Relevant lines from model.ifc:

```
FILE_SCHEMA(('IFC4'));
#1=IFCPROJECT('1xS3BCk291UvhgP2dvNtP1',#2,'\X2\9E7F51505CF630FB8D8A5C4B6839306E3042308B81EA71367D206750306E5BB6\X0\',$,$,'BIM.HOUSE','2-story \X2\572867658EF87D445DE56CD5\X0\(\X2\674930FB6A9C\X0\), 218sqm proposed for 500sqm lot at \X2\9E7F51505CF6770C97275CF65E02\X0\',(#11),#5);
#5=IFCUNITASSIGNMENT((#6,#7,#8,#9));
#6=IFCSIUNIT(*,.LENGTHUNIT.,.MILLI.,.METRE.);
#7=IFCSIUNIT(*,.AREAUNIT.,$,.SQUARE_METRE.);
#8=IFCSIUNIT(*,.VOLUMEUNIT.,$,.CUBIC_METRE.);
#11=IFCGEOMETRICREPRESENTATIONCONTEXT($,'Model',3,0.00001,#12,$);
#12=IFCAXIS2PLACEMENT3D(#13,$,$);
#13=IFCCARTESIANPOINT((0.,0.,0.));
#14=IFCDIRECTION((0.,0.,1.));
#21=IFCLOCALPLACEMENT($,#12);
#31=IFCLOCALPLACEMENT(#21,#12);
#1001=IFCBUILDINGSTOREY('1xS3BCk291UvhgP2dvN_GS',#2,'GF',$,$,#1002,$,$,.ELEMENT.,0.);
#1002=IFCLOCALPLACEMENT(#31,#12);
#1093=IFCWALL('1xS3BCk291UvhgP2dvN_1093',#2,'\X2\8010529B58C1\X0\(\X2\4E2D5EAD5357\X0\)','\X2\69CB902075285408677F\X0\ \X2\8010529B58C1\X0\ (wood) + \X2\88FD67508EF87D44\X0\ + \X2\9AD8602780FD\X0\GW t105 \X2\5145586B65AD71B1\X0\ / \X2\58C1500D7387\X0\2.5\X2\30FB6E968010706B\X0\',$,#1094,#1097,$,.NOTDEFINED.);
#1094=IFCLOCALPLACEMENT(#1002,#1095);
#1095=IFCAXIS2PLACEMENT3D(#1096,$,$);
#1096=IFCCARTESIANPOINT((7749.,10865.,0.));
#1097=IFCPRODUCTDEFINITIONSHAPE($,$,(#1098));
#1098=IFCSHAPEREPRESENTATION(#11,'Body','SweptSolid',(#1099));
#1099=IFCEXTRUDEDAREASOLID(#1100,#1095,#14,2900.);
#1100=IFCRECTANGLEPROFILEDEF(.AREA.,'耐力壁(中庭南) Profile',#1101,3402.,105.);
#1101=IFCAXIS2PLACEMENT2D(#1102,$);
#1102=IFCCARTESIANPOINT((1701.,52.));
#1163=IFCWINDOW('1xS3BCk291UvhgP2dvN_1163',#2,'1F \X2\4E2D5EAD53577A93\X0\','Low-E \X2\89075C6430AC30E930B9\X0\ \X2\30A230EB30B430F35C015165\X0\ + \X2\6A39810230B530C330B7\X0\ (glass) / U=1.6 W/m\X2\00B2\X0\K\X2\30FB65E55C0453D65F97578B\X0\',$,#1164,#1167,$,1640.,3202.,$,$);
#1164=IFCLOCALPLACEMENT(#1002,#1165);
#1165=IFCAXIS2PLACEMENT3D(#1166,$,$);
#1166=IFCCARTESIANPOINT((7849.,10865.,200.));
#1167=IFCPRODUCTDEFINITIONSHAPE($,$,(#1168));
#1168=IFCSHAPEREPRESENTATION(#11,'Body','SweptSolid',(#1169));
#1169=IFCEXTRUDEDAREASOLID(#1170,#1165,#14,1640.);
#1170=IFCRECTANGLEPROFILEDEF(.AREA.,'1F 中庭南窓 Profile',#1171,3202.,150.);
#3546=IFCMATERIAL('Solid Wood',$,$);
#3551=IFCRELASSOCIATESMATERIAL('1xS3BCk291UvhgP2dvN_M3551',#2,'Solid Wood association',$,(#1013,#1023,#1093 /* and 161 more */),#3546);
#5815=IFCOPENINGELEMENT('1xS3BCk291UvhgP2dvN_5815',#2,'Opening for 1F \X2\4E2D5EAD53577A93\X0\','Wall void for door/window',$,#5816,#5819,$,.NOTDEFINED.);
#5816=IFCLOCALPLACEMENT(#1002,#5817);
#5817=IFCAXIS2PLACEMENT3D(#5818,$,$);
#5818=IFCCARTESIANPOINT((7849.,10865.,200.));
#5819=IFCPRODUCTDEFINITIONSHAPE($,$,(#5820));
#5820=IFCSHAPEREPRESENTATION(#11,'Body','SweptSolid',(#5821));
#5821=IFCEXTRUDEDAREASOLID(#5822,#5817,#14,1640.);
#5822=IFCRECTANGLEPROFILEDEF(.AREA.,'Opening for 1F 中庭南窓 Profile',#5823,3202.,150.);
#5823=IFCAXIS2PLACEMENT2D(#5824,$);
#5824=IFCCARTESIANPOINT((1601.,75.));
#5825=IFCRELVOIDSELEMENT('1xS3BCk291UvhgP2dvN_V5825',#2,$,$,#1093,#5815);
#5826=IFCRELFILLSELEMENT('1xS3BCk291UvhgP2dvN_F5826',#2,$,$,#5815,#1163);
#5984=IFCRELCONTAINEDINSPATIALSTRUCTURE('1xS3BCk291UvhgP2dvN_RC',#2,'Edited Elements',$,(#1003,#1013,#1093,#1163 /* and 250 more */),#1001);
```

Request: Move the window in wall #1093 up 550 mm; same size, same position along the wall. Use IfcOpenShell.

```python
import numpy as np
import ifcopenshell
import ifcopenshell.api.geometry
import ifcopenshell.util.placement
import ifcopenshell.util.unit

model = ifcopenshell.open("model.ifc")
unit_scale = ifcopenshell.util.unit.calculate_unit_scale(model)

window = model.by_guid("1xS3BCk291UvhgP2dvN_1163")
opening = window.FillsVoids[0].RelatingOpeningElement
dz = 550.0

shift = np.array([0.0, 0.0, dz])
# The window is not placed relative to its opening, so move both.
for product in (opening, window):
    matrix = ifcopenshell.util.placement.get_local_placement(product.ObjectPlacement)
    matrix[:3, 3] += shift
    ifcopenshell.api.geometry.edit_object_placement(model, product=product, matrix=matrix, is_si=False)

print(f"moved by {dz * unit_scale:+.3f} m")

model.write("model_updated.ifc")
```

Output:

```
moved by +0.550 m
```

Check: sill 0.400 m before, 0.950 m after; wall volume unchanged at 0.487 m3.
